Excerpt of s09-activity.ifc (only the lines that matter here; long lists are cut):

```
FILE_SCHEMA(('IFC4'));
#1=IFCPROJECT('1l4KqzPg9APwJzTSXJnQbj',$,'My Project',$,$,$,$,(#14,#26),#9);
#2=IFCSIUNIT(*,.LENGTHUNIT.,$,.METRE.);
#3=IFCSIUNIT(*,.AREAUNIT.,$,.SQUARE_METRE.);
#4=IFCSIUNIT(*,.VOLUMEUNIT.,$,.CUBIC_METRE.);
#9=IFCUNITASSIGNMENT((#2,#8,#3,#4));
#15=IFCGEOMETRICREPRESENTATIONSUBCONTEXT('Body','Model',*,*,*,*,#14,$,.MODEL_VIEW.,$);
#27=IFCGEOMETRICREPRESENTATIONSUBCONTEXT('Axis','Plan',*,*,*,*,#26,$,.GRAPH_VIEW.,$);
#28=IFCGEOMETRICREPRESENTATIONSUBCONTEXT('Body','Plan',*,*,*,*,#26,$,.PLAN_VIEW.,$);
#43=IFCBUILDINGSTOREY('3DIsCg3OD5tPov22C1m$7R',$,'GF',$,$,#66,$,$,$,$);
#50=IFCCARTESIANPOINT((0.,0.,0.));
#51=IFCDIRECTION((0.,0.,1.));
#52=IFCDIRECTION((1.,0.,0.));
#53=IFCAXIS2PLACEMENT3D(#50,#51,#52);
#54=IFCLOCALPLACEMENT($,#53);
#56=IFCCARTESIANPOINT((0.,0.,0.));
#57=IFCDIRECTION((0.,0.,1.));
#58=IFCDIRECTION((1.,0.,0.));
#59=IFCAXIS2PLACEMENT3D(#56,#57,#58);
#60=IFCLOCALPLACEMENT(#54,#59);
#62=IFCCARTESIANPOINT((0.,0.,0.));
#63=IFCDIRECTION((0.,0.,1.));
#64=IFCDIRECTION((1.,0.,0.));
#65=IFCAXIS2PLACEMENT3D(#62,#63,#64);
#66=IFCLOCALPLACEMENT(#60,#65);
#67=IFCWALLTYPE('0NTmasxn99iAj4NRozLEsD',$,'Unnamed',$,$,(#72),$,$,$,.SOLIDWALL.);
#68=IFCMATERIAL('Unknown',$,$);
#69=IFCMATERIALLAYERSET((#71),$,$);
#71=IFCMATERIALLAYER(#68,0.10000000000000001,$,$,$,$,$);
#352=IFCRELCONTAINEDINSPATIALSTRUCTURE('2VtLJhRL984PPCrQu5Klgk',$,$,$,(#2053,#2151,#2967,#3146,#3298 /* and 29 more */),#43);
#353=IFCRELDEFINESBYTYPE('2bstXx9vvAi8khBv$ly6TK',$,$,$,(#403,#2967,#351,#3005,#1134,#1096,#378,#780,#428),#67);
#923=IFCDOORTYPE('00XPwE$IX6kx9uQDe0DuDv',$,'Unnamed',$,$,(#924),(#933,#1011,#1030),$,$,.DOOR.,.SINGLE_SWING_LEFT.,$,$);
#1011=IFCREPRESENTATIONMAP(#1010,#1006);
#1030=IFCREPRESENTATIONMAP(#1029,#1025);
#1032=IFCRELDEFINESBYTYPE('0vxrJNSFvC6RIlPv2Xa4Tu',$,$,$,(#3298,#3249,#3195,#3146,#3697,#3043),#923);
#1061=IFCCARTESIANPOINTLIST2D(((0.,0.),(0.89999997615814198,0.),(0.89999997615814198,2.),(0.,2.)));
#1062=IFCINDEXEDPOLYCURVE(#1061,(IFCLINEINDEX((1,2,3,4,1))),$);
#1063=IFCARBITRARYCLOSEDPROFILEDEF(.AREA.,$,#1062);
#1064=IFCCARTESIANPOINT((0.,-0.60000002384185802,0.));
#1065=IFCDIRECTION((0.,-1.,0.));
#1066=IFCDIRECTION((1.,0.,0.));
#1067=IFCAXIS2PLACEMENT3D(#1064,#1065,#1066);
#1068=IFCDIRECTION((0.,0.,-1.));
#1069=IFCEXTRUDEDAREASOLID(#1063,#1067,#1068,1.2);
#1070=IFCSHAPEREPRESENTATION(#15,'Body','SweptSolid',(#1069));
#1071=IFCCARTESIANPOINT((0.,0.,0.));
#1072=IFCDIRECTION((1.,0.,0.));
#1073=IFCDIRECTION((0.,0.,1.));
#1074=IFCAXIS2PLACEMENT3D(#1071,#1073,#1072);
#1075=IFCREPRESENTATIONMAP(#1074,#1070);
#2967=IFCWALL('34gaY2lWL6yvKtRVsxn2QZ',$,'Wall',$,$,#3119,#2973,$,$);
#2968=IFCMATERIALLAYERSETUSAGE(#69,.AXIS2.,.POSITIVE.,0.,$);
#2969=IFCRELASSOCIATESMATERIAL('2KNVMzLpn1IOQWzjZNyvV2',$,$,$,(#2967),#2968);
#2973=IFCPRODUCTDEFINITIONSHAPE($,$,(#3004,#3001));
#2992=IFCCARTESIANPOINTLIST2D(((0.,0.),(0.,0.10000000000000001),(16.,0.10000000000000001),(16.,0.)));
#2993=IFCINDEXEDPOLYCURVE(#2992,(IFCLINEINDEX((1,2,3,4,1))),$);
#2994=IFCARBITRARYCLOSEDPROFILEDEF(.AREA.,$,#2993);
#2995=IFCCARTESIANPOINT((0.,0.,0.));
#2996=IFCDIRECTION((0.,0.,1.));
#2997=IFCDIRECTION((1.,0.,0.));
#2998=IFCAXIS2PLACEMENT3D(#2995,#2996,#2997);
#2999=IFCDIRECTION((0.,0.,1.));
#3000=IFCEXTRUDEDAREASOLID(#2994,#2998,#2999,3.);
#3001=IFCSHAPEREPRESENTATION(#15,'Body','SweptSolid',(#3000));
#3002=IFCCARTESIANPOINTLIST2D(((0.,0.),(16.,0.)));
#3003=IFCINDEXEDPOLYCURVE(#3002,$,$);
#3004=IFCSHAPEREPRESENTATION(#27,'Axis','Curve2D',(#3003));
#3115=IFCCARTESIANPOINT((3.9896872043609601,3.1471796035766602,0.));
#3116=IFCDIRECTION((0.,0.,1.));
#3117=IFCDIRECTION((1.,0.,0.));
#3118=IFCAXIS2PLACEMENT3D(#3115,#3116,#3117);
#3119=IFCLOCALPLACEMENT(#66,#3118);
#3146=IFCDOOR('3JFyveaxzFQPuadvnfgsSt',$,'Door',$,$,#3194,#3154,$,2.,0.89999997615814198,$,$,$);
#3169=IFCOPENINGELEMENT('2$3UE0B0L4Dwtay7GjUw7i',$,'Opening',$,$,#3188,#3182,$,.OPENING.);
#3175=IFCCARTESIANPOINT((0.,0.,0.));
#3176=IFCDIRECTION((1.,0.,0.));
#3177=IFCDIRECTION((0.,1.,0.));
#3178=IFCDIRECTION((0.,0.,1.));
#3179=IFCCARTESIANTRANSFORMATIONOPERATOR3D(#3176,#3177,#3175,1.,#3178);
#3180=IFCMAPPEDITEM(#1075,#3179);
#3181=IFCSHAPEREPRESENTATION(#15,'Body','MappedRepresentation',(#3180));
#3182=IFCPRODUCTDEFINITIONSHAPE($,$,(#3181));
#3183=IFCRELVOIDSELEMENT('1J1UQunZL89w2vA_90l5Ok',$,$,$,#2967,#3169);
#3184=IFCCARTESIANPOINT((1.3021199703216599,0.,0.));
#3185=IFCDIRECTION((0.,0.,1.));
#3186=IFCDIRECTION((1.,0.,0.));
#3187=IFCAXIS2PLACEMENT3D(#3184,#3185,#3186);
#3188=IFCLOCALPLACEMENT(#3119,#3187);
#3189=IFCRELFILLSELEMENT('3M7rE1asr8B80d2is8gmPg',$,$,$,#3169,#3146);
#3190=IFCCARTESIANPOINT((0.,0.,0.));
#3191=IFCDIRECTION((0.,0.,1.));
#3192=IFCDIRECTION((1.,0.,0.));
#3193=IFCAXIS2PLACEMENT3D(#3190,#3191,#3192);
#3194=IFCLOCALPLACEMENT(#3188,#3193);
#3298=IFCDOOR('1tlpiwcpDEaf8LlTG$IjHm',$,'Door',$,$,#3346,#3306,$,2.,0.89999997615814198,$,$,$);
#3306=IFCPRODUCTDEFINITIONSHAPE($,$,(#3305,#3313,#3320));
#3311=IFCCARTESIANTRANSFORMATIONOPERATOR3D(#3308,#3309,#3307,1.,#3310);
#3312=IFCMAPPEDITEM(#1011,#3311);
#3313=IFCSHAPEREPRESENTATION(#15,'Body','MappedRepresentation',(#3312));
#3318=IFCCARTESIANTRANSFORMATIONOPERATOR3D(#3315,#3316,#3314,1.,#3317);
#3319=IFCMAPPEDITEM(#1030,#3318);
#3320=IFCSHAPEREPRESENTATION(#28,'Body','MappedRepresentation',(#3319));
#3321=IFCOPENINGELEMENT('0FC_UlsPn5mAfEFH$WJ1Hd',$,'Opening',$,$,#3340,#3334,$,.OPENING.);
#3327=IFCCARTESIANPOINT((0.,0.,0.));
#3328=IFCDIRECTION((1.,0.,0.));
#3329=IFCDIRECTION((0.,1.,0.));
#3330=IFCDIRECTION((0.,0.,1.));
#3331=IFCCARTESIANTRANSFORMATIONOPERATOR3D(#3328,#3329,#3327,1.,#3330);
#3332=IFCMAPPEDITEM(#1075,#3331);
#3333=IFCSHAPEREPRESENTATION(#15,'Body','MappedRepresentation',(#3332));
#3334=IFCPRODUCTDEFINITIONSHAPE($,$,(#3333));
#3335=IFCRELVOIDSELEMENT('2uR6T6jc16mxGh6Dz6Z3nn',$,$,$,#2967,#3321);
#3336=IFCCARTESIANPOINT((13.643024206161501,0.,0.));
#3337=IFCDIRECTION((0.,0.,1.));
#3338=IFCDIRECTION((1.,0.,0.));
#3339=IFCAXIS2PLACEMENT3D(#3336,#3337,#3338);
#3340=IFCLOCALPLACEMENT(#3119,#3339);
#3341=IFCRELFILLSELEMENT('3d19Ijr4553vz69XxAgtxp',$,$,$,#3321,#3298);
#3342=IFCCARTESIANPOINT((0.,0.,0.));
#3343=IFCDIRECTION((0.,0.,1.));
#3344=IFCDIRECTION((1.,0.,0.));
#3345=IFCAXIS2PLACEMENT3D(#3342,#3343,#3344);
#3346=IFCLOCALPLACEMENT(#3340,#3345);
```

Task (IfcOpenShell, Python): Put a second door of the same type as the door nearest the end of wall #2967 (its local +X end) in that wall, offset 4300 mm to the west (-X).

```python
import ifcopenshell
import ifcopenshell.api.feature
import ifcopenshell.api.geometry
import ifcopenshell.api.root
import ifcopenshell.geom
import ifcopenshell.util.element
import ifcopenshell.util.placement
import ifcopenshell.util.shape
import ifcopenshell.util.unit

model = ifcopenshell.open("s09-activity.ifc")
unit_scale = ifcopenshell.util.unit.calculate_unit_scale(model)
settings = ifcopenshell.geom.settings()


def volume(element):
    """Net volume in cubic metres, openings subtracted."""
    shape = ifcopenshell.geom.create_shape(settings, element)
    return ifcopenshell.util.shape.get_volume(shape.geometry)


door = model.by_guid("1tlpiwcpDEaf8LlTG$IjHm")
opening = door.FillsVoids[0].RelatingOpeningElement
wall = opening.VoidsElements[0].RelatingBuildingElement
before = volume(wall)
shift = ifcopenshell.util.placement.get_local_placement(wall.ObjectPlacement)[:3, 0] * -4.3 / unit_scale

# copy_class copies the void relationship, type, container and properties, but no geometry.
new_opening = ifcopenshell.api.root.copy_class(model, product=opening)
new_opening.Representation = ifcopenshell.util.element.copy_deep(
    model, opening.Representation, exclude=["IfcGeometricRepresentationContext", "IfcRepresentationMap"]
)
new_door = ifcopenshell.api.root.copy_class(model, product=door)
new_door.Representation = ifcopenshell.util.element.copy_deep(
    model, door.Representation, exclude=["IfcGeometricRepresentationContext", "IfcRepresentationMap"]
)
ifcopenshell.api.feature.add_filling(model, opening=new_opening, element=new_door)

for old, new in ((opening, new_opening), (door, new_door)):
    matrix = ifcopenshell.util.placement.get_local_placement(old.ObjectPlacement)
    matrix[:3, 3] += shift
    ifcopenshell.api.geometry.edit_object_placement(model, product=new, matrix=matrix, is_si=False)

after = volume(wall)

print(f"wall volume {before:.3f} -> {after:.3f} m3")

model.write("s09-activity_updated.ifc")
```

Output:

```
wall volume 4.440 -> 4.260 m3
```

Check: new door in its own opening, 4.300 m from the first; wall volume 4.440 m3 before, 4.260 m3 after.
